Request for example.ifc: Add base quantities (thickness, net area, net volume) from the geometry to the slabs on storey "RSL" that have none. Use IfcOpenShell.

First a look at what the model holds.

```python
import ifcopenshell
import ifcopenshell.util.element
import ifcopenshell.util.unit

model = ifcopenshell.open("example.ifc")
print(model.schema)
for unit_type in ("LENGTHUNIT", "AREAUNIT", "VOLUMEUNIT"):
    print(unit_type, ifcopenshell.util.unit.calculate_unit_scale(model, unit_type))
storey = next(s for s in model.by_type("IfcBuildingStorey") if s.Name == "RSL")
slabs = [e for e in ifcopenshell.util.element.get_decomposition(storey) if e.is_a("IfcSlab")]
for e in sorted(slabs, key=lambda e: e.id()):
    print(e.id(), e.is_a(), e.Name, list(ifcopenshell.util.element.get_psets(e, qtos_only=True)), sep=" | ")
```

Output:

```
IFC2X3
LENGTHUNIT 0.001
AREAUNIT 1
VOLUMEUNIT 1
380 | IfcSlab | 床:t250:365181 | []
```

```python
import ifcopenshell
import ifcopenshell.api.pset
import ifcopenshell.geom
import ifcopenshell.util.element
import ifcopenshell.util.shape
import ifcopenshell.util.unit

model = ifcopenshell.open("example.ifc")
unit_scale = ifcopenshell.util.unit.calculate_unit_scale(model)
area_scale = ifcopenshell.util.unit.calculate_unit_scale(model, "AREAUNIT")
volume_scale = ifcopenshell.util.unit.calculate_unit_scale(model, "VOLUMEUNIT")
settings = ifcopenshell.geom.settings()

storey = next(s for s in model.by_type("IfcBuildingStorey") if s.Name == "RSL")
slabs = [e for e in ifcopenshell.util.element.get_decomposition(storey) if e.is_a("IfcSlab")]

for e in sorted(slabs, key=lambda e: e.id()):
    if ifcopenshell.util.element.get_psets(e, qtos_only=True, should_inherit=False):
        continue
    # Geometry comes back in metres, in the element's own axes.
    shape = ifcopenshell.geom.create_shape(settings, e)
    values = {
        "Width": ifcopenshell.util.shape.get_z(shape.geometry) / unit_scale,
        "NetArea": ifcopenshell.util.shape.get_footprint_area(shape.geometry) / area_scale,
        "NetVolume": ifcopenshell.util.shape.get_volume(shape.geometry) / volume_scale,
    }
    qto = ifcopenshell.api.pset.add_qto(model, product=e, name="BaseQuantities")
    ifcopenshell.api.pset.edit_qto(model, qto=qto, properties=values)
    print(e.id(), {k: round(v, 3) for k, v in values.items()})

model.write("example_v2.ifc")
```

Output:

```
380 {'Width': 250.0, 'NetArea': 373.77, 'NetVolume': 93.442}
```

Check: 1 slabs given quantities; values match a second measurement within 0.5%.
